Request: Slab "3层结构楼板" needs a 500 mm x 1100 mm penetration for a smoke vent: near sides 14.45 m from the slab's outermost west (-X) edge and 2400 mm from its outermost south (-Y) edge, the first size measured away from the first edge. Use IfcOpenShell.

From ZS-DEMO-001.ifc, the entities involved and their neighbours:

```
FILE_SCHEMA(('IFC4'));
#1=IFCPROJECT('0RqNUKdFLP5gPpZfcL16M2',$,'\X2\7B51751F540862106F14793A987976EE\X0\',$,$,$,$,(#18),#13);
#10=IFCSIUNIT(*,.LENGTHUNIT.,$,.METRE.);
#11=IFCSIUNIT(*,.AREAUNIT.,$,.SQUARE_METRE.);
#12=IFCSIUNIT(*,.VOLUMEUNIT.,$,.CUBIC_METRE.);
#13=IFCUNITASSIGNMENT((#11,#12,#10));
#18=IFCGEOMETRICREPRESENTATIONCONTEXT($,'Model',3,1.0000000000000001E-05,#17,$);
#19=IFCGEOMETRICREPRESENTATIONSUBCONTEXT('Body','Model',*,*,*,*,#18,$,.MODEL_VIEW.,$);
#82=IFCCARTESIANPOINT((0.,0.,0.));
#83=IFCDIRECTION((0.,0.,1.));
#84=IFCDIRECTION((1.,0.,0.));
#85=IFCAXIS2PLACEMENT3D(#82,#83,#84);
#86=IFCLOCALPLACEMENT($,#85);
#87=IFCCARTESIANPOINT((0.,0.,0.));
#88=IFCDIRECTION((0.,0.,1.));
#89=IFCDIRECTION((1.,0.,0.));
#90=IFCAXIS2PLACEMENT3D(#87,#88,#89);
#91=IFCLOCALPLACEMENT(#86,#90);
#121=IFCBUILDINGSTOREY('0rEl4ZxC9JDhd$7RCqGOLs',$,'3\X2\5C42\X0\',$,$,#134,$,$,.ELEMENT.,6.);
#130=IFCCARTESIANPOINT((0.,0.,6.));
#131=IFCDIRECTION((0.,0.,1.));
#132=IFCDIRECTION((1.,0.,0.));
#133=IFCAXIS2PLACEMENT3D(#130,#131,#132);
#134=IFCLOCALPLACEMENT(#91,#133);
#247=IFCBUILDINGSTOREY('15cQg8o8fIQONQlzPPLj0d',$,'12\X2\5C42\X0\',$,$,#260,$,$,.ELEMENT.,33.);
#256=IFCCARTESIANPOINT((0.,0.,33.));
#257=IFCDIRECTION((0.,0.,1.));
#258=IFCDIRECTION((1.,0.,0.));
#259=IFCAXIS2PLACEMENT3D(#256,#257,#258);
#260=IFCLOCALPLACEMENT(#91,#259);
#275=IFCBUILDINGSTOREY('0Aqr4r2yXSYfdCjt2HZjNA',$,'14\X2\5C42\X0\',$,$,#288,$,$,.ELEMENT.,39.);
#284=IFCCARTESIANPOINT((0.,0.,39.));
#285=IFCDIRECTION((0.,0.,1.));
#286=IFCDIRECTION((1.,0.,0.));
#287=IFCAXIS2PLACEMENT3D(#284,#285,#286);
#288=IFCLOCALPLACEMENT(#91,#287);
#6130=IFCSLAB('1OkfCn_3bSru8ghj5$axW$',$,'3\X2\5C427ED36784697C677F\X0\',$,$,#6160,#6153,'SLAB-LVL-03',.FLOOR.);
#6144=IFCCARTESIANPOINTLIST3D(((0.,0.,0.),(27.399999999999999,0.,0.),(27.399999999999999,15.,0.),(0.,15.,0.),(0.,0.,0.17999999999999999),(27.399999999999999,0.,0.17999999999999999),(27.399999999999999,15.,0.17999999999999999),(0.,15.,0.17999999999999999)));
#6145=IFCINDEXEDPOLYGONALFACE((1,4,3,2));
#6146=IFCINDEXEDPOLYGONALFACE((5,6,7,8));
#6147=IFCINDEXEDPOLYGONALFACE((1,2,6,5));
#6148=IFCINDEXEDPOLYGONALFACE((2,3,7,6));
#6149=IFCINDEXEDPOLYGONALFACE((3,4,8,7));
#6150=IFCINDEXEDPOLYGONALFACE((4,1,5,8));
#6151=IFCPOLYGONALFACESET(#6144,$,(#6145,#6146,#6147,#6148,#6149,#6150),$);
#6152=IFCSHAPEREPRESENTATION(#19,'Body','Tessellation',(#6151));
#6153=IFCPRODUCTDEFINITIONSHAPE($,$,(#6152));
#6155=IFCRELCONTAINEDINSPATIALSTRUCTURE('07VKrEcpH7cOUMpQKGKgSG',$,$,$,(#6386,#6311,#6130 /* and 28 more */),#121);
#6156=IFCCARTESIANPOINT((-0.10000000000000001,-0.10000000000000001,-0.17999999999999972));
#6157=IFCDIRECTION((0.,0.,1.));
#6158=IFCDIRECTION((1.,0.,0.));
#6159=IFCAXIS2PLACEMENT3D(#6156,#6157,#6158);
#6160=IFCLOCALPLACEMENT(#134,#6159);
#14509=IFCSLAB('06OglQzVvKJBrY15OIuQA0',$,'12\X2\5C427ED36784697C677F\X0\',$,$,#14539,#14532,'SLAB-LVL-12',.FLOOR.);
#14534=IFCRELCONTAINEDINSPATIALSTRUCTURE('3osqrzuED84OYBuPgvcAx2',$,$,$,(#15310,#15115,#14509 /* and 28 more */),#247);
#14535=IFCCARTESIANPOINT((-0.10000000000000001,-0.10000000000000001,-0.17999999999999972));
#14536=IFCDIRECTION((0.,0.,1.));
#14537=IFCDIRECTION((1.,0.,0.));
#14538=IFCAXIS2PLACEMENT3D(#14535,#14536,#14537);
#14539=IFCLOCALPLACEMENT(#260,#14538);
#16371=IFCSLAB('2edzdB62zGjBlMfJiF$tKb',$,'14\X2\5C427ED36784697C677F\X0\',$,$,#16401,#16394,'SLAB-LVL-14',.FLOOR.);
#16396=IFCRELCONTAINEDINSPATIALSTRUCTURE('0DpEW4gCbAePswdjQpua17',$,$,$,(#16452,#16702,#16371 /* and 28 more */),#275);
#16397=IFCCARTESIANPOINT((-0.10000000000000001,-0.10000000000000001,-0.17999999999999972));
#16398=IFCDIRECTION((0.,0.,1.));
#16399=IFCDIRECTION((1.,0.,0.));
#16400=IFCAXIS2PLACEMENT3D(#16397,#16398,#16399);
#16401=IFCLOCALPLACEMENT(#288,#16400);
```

```python
import numpy as np
import ifcopenshell
import ifcopenshell.api.feature
import ifcopenshell.api.geometry
import ifcopenshell.api.root
import ifcopenshell.geom
import ifcopenshell.util.placement
import ifcopenshell.util.representation
import ifcopenshell.util.shape
import ifcopenshell.util.unit

model = ifcopenshell.open("ZS-DEMO-001.ifc")
unit_scale = ifcopenshell.util.unit.calculate_unit_scale(model)
settings = ifcopenshell.geom.settings()


def volume(element):
    """Net volume in cubic metres, openings subtracted."""
    shape = ifcopenshell.geom.create_shape(settings, element)
    return ifcopenshell.util.shape.get_volume(shape.geometry)


slab = model.by_id(6130)
before = volume(slab)

# Extent in the slab's own axes, in metres. The edges named are its -X and -Y sides.
slab_shape = ifcopenshell.geom.create_shape(settings, slab)
vertices = ifcopenshell.util.shape.get_vertices(slab_shape.geometry)
x_min, y_min, bottom = vertices.min(axis=0)
top = vertices[:, 2].max()

opening = ifcopenshell.api.root.create_entity(model, ifc_class="IfcOpeningElement", name="Smoke vent opening", predefined_type="OPENING")
context = ifcopenshell.util.representation.get_context(model, "Model", "Body", "MODEL_VIEW")
width, depth = 0.5, 1.1
outline = [(0.0, 0.0), (width, 0.0), (width, depth), (0.0, depth), (0.0, 0.0)]
# Overshoot both faces by 50 mm so the cut is clean.
shape = ifcopenshell.api.geometry.add_slab_representation(
    model, context=context, depth=top - bottom + 0.1, polyline=outline
)
ifcopenshell.api.geometry.assign_representation(model, product=opening, representation=shape)

matrix = ifcopenshell.util.placement.get_local_placement(slab.ObjectPlacement)
matrix[:, 3] = matrix @ np.append(np.array([x_min + 14.45, y_min + 2.4, bottom - 0.05]) / unit_scale, 1.0)
ifcopenshell.api.geometry.edit_object_placement(model, product=opening, matrix=matrix, is_si=False)
ifcopenshell.api.feature.add_feature(model, feature=opening, element=slab)

after = volume(slab)

print(f"slab volume {before:.3f} -> {after:.3f} m3")

model.write("ZS-DEMO-001-out.ifc")
```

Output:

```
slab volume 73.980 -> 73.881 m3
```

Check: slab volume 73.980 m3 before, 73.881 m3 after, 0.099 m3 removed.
